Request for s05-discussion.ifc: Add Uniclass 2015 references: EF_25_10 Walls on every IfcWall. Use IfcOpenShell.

First a look at what the model holds.

```python
import ifcopenshell

model = ifcopenshell.open("s05-discussion.ifc")
print(model.schema)
print("classifications:", [c.Name for c in model.by_type("IfcClassification")])
for ifc_class in ("IfcDoor", "IfcRoof", "IfcStair", "IfcWall", "IfcWindow"):
    print(ifc_class, len(model.by_type(ifc_class)))
```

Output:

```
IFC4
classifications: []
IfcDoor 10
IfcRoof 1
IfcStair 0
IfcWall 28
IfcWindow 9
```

```python
import ifcopenshell
import ifcopenshell.api.classification

model = ifcopenshell.open("s05-discussion.ifc")

system = ifcopenshell.api.classification.add_classification(model, classification="Uniclass 2015")

codes = {
    "IfcWall": ("EF_25_10", "Walls"),
}
for ifc_class, (code, name) in codes.items():
    products = model.by_type(ifc_class)
    ifcopenshell.api.classification.add_reference(
        model, products=products, classification=system, identification=code, name=name
    )
    print(code, len(products))

model.write("s05-discussion-out.ifc")
```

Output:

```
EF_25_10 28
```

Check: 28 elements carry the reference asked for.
